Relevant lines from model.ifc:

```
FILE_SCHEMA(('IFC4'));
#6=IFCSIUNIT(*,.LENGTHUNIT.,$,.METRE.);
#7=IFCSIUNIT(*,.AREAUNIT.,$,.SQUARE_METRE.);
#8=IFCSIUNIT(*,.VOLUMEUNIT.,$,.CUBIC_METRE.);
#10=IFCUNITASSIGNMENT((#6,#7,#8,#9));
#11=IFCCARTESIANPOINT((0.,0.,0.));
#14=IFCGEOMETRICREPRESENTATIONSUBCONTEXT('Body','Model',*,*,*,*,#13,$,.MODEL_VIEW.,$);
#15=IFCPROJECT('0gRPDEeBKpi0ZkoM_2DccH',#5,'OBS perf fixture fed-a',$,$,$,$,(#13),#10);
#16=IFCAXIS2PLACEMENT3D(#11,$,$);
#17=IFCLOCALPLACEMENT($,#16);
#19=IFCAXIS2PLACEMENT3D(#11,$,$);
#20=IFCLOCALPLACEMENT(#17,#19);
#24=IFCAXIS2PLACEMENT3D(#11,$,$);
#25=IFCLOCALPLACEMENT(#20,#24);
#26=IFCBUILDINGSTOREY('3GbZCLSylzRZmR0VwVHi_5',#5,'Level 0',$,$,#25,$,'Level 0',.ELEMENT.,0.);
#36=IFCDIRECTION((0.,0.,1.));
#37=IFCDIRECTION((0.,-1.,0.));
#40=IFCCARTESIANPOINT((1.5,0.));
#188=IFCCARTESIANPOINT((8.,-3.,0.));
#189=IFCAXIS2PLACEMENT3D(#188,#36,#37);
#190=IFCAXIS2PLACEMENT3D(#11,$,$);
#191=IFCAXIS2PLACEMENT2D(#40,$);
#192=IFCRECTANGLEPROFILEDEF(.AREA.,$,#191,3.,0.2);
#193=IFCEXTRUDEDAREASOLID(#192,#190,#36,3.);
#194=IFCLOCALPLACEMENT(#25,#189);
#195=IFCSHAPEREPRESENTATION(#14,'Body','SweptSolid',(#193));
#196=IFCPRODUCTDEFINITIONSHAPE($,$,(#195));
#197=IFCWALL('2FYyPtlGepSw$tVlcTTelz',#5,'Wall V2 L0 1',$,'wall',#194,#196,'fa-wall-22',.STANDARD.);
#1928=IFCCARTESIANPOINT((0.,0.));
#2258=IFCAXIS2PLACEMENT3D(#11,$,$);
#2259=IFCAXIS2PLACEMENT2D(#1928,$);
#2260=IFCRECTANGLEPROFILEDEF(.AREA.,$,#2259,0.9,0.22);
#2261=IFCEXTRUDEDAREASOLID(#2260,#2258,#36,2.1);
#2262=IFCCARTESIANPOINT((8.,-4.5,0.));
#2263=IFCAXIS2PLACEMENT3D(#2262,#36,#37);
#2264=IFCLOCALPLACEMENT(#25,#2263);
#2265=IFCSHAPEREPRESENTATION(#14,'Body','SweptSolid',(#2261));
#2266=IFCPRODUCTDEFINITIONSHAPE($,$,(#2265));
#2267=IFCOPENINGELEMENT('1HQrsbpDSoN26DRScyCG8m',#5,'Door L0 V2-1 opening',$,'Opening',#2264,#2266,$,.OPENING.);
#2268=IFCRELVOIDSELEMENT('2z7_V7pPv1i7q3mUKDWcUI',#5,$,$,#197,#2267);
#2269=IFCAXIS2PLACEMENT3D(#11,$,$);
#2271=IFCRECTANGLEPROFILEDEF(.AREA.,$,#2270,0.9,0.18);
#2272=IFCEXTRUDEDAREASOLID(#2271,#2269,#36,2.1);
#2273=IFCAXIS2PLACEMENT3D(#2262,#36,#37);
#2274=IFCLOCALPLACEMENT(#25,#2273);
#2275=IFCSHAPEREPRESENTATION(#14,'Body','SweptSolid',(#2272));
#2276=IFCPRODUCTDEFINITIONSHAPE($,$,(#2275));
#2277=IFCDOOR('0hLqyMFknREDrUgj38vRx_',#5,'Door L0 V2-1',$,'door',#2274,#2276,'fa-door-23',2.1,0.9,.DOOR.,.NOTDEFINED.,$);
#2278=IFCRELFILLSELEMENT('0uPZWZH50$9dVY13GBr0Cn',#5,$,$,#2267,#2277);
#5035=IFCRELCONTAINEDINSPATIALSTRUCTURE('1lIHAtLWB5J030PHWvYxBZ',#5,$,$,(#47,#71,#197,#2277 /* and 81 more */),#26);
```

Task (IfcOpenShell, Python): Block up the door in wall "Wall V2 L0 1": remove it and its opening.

```python
import ifcopenshell
import ifcopenshell.api.feature
import ifcopenshell.api.root
import ifcopenshell.geom
import ifcopenshell.util.shape

model = ifcopenshell.open("model.ifc")
settings = ifcopenshell.geom.settings()


def volume(element):
    """Net volume in cubic metres, openings subtracted."""
    shape = ifcopenshell.geom.create_shape(settings, element)
    return ifcopenshell.util.shape.get_volume(shape.geometry)


door = model.by_id(2277)
opening = door.FillsVoids[0].RelatingOpeningElement
wall = opening.VoidsElements[0].RelatingBuildingElement
before = volume(wall)

ifcopenshell.api.root.remove_product(model, product=door)
ifcopenshell.api.feature.remove_feature(model, feature=opening)

after = volume(wall)

print(f"wall volume {before:.3f} -> {after:.3f} m3")

model.write("model_updated.ifc")
```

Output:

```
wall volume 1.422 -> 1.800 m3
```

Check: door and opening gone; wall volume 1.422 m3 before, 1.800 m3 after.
